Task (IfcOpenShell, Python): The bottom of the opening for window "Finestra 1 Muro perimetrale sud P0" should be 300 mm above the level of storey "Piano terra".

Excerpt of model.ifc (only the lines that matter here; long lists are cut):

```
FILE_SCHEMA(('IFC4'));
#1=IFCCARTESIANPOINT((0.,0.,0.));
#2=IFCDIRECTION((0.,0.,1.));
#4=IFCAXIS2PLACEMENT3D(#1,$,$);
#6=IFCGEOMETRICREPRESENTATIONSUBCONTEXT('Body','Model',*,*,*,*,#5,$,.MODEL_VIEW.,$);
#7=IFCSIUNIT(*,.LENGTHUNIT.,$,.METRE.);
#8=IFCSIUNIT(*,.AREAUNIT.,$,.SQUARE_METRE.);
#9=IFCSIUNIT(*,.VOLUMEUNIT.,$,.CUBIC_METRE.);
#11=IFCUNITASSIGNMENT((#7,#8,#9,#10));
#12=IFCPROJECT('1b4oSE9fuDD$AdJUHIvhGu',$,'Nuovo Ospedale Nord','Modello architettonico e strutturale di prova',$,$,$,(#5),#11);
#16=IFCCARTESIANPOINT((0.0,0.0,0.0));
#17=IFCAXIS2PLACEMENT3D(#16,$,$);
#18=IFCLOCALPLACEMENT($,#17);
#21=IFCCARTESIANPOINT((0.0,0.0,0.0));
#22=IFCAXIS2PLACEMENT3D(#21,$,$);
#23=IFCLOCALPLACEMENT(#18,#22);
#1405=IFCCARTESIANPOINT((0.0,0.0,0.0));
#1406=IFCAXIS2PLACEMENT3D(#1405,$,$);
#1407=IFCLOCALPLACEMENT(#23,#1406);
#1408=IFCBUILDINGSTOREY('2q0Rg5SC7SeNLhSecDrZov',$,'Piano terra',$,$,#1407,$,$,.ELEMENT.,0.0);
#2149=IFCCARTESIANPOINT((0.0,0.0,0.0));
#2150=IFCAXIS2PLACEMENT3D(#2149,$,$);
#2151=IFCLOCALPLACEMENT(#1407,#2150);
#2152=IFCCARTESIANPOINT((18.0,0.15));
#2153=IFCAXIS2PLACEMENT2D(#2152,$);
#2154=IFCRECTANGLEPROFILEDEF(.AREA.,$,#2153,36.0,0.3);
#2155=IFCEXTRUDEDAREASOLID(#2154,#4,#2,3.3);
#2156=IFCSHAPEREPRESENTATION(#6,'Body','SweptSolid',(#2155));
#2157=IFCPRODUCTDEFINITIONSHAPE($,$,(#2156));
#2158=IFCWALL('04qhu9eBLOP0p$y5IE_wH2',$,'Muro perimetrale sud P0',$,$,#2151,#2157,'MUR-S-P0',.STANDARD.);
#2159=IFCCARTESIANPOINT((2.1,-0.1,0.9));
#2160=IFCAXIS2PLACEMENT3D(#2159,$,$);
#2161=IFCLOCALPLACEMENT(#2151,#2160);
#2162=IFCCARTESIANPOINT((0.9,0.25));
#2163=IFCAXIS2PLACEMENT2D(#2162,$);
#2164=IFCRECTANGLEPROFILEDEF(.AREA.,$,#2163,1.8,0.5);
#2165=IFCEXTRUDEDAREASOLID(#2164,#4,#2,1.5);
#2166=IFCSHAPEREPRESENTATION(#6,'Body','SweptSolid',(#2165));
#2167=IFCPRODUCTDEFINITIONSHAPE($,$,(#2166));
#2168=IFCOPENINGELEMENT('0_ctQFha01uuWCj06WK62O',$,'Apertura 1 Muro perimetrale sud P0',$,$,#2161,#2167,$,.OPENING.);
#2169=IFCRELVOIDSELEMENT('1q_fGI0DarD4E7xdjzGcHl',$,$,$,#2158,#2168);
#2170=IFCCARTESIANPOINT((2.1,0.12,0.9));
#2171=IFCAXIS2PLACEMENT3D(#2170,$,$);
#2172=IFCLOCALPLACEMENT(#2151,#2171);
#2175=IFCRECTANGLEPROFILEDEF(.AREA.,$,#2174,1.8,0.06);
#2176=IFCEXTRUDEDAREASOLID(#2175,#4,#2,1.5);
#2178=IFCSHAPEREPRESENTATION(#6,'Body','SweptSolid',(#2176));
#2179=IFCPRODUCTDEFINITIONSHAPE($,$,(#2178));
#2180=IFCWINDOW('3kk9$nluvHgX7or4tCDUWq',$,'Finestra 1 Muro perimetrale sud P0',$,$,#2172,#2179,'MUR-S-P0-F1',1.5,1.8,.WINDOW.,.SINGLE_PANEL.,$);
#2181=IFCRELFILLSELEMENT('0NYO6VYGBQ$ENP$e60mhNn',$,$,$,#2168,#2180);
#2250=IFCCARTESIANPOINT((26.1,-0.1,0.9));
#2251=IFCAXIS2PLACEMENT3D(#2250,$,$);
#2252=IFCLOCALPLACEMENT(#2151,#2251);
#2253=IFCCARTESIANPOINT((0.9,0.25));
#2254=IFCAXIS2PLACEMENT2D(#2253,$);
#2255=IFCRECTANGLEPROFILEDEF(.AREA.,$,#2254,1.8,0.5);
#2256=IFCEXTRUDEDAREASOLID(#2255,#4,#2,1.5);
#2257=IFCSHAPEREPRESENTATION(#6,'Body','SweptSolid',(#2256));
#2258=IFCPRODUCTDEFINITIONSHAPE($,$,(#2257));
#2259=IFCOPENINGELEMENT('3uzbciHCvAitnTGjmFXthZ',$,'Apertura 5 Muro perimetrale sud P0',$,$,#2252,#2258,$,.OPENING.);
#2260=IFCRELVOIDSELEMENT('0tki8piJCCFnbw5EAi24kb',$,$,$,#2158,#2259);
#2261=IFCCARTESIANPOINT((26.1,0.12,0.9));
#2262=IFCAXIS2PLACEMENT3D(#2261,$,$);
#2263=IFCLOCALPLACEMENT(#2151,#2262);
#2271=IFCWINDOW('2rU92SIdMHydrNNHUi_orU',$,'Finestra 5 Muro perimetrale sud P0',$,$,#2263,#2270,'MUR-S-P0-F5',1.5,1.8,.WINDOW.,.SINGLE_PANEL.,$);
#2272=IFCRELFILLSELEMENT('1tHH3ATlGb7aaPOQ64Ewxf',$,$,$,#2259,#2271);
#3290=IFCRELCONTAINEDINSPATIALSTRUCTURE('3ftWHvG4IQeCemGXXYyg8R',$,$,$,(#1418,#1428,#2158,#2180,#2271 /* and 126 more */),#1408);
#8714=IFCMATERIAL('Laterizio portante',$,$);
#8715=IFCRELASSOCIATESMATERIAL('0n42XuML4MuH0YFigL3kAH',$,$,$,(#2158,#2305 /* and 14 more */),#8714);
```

```python
import numpy as np
import ifcopenshell
import ifcopenshell.api.geometry
import ifcopenshell.geom
import ifcopenshell.util.element
import ifcopenshell.util.placement
import ifcopenshell.util.shape
import ifcopenshell.util.unit

model = ifcopenshell.open("model.ifc")
unit_scale = ifcopenshell.util.unit.calculate_unit_scale(model)

window = model.by_guid("3kk9$nluvHgX7or4tCDUWq")
opening = window.FillsVoids[0].RelatingOpeningElement
storey = ifcopenshell.util.element.get_container(window, ifc_class="IfcBuildingStorey")
level = ifcopenshell.util.placement.get_local_placement(storey.ObjectPlacement)[2, 3]

# The opening's origin need not be at the sill, so measure its lowest point.
shape = ifcopenshell.geom.create_shape(ifcopenshell.geom.settings(), opening)
bottom = ifcopenshell.util.shape.get_shape_bottom_elevation(shape, shape.geometry) / unit_scale
dz = level + 0.3 - bottom

shift = np.array([0.0, 0.0, dz])
# The window is not placed relative to its opening, so move both.
for product in (opening, window):
    matrix = ifcopenshell.util.placement.get_local_placement(product.ObjectPlacement)
    matrix[:3, 3] += shift
    ifcopenshell.api.geometry.edit_object_placement(model, product=product, matrix=matrix, is_si=False)

print(f"moved by {dz * unit_scale:+.3f} m")

model.write("model_edited.ifc")
```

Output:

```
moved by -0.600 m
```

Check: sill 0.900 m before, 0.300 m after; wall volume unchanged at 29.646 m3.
